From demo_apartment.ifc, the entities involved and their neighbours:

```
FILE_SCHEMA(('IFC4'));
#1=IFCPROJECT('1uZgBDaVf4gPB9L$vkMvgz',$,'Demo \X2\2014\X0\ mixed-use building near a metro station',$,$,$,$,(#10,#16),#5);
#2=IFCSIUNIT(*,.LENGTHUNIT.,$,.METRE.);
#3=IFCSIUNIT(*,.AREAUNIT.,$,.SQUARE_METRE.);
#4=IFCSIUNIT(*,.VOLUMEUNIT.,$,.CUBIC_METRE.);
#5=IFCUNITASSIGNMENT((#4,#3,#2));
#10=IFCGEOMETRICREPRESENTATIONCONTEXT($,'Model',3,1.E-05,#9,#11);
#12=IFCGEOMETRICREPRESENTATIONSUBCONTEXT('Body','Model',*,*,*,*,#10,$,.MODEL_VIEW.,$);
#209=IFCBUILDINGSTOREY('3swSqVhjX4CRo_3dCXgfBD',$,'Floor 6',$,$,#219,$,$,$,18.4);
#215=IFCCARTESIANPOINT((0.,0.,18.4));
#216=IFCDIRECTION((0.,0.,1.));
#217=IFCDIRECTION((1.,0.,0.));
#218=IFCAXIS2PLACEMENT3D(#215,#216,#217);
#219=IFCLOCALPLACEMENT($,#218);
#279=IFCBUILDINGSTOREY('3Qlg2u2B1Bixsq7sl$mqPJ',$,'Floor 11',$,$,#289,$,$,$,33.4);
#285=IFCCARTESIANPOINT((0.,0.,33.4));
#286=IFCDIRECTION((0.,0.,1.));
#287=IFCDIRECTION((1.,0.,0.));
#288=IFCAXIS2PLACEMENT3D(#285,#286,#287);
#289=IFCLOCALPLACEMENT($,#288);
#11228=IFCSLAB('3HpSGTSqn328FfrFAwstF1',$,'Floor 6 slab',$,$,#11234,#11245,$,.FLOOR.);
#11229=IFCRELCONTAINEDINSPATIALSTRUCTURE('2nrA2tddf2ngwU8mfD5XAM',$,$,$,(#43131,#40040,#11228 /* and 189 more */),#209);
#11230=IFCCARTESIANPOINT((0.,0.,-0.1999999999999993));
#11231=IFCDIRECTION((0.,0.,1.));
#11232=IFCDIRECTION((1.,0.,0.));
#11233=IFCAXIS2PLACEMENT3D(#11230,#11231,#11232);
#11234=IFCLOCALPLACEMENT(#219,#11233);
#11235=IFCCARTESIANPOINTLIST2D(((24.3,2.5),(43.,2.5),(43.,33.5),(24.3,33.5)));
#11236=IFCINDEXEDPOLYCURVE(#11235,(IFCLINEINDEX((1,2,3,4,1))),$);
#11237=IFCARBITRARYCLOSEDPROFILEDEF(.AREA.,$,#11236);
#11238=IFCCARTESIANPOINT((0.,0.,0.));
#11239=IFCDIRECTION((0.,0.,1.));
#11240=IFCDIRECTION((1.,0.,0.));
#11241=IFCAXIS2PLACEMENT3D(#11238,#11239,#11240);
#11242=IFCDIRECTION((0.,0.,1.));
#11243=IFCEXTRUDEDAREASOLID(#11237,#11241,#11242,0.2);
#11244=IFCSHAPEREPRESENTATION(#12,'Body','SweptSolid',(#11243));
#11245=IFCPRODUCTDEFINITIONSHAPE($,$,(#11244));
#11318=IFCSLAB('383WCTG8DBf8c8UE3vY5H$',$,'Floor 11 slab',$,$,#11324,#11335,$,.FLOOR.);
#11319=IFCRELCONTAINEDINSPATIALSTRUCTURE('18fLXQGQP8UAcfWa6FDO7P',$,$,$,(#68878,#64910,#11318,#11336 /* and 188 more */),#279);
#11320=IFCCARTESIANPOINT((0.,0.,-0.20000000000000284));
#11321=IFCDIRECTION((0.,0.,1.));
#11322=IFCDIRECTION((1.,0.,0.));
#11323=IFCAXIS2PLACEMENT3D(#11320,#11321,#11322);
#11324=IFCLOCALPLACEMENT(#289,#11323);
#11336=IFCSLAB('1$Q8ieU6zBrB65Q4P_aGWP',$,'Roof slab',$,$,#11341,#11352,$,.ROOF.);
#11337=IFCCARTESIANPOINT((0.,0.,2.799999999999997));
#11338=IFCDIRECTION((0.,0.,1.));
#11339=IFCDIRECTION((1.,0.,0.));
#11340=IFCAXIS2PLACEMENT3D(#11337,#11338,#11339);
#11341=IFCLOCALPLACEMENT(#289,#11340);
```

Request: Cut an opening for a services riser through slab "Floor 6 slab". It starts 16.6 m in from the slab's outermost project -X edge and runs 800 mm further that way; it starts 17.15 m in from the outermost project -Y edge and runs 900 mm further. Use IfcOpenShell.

```python
import numpy as np
import ifcopenshell
import ifcopenshell.api.feature
import ifcopenshell.api.geometry
import ifcopenshell.api.root
import ifcopenshell.geom
import ifcopenshell.util.placement
import ifcopenshell.util.representation
import ifcopenshell.util.shape
import ifcopenshell.util.unit

model = ifcopenshell.open("demo_apartment.ifc")
unit_scale = ifcopenshell.util.unit.calculate_unit_scale(model)
settings = ifcopenshell.geom.settings()


def volume(element):
    """Net volume in cubic metres, openings subtracted."""
    shape = ifcopenshell.geom.create_shape(settings, element)
    return ifcopenshell.util.shape.get_volume(shape.geometry)


slab = model.by_id(11228)
before = volume(slab)

# Extent in the slab's own axes, in metres. The edges named are its -X and -Y sides.
slab_shape = ifcopenshell.geom.create_shape(settings, slab)
vertices = ifcopenshell.util.shape.get_vertices(slab_shape.geometry)
x_min, y_min, bottom = vertices.min(axis=0)
top = vertices[:, 2].max()

opening = ifcopenshell.api.root.create_entity(model, ifc_class="IfcOpeningElement", name="Services riser opening", predefined_type="OPENING")
context = ifcopenshell.util.representation.get_context(model, "Model", "Body", "MODEL_VIEW")
width, depth = 0.8, 0.9
outline = [(0.0, 0.0), (width, 0.0), (width, depth), (0.0, depth), (0.0, 0.0)]
# Overshoot both faces by 50 mm so the cut is clean.
shape = ifcopenshell.api.geometry.add_slab_representation(
    model, context=context, depth=top - bottom + 0.1, polyline=outline
)
ifcopenshell.api.geometry.assign_representation(model, product=opening, representation=shape)

matrix = ifcopenshell.util.placement.get_local_placement(slab.ObjectPlacement)
matrix[:, 3] = matrix @ np.append(np.array([x_min + 16.6, y_min + 17.15, bottom - 0.05]) / unit_scale, 1.0)
ifcopenshell.api.geometry.edit_object_placement(model, product=opening, matrix=matrix, is_si=False)
ifcopenshell.api.feature.add_feature(model, feature=opening, element=slab)

after = volume(slab)

print(f"slab volume {before:.3f} -> {after:.3f} m3")

model.write("demo_apartment_updated.ifc")
```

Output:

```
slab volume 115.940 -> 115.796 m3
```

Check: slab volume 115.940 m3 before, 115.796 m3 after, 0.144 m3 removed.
